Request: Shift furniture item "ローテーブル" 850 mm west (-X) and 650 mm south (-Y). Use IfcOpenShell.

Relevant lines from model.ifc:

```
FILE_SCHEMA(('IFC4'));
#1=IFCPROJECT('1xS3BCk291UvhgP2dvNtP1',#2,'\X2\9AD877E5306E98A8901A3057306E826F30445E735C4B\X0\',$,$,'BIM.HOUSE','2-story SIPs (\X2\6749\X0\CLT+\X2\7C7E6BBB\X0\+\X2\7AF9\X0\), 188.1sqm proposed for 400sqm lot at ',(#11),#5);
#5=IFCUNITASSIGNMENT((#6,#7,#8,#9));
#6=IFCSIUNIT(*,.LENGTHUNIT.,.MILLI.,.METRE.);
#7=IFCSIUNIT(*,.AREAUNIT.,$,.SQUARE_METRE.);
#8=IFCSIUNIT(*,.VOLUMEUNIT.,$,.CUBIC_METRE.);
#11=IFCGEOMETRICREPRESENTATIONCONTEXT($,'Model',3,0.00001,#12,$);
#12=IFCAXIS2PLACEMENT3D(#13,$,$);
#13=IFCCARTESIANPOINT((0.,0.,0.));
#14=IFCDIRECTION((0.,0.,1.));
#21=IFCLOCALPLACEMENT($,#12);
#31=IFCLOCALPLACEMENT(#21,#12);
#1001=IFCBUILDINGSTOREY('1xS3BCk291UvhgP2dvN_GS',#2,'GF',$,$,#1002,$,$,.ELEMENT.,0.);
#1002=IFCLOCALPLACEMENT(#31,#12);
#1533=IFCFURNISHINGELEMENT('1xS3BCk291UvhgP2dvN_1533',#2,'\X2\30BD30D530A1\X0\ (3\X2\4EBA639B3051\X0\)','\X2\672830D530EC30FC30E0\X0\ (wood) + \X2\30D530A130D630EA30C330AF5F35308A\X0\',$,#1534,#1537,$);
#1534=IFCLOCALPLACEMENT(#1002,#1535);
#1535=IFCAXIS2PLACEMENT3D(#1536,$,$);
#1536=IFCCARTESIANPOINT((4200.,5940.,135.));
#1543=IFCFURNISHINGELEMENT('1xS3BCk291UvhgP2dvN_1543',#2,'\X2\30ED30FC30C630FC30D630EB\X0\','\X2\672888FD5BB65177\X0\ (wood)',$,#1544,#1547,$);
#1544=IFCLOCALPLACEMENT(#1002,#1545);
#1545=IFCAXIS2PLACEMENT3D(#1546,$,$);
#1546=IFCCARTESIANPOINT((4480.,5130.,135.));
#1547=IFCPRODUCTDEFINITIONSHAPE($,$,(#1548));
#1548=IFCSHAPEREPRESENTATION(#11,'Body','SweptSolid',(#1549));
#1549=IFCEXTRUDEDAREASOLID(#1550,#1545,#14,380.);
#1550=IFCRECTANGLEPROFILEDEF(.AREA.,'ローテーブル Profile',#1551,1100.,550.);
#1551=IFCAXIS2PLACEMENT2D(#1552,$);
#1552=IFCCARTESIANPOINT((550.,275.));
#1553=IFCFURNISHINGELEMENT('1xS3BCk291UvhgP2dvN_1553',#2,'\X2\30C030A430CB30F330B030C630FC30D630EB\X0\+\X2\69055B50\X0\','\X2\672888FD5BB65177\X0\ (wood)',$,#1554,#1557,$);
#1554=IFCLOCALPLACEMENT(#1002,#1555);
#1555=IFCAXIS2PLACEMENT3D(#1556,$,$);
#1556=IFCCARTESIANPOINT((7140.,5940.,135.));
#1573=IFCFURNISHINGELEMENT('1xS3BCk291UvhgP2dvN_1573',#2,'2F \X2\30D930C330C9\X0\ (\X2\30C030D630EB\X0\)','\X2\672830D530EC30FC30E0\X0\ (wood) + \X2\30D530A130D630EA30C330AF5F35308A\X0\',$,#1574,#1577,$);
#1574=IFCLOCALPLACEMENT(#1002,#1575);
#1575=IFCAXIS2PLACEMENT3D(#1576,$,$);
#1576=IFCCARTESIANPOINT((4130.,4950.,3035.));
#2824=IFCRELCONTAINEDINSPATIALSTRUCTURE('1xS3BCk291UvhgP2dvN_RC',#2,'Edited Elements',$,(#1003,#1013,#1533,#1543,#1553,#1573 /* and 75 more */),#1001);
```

```python
import ifcopenshell
import ifcopenshell.api.geometry
import ifcopenshell.util.placement
import ifcopenshell.util.unit

model = ifcopenshell.open("model.ifc")
unit_scale = ifcopenshell.util.unit.calculate_unit_scale(model)

item = model.by_guid("1xS3BCk291UvhgP2dvN_1543")
matrix = ifcopenshell.util.placement.get_local_placement(item.ObjectPlacement)
matrix[0, 3] -= 0.85 / unit_scale
matrix[1, 3] -= 0.65 / unit_scale
ifcopenshell.api.geometry.edit_object_placement(model, product=item, matrix=matrix, is_si=False)

print(ifcopenshell.util.placement.get_local_placement(item.ObjectPlacement).round(3) + 0.0)

model.write("model_rev.ifc")
```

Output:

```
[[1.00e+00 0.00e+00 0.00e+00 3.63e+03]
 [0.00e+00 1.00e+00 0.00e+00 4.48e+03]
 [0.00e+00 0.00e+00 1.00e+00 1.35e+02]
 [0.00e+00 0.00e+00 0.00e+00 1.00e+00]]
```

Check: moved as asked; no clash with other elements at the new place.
